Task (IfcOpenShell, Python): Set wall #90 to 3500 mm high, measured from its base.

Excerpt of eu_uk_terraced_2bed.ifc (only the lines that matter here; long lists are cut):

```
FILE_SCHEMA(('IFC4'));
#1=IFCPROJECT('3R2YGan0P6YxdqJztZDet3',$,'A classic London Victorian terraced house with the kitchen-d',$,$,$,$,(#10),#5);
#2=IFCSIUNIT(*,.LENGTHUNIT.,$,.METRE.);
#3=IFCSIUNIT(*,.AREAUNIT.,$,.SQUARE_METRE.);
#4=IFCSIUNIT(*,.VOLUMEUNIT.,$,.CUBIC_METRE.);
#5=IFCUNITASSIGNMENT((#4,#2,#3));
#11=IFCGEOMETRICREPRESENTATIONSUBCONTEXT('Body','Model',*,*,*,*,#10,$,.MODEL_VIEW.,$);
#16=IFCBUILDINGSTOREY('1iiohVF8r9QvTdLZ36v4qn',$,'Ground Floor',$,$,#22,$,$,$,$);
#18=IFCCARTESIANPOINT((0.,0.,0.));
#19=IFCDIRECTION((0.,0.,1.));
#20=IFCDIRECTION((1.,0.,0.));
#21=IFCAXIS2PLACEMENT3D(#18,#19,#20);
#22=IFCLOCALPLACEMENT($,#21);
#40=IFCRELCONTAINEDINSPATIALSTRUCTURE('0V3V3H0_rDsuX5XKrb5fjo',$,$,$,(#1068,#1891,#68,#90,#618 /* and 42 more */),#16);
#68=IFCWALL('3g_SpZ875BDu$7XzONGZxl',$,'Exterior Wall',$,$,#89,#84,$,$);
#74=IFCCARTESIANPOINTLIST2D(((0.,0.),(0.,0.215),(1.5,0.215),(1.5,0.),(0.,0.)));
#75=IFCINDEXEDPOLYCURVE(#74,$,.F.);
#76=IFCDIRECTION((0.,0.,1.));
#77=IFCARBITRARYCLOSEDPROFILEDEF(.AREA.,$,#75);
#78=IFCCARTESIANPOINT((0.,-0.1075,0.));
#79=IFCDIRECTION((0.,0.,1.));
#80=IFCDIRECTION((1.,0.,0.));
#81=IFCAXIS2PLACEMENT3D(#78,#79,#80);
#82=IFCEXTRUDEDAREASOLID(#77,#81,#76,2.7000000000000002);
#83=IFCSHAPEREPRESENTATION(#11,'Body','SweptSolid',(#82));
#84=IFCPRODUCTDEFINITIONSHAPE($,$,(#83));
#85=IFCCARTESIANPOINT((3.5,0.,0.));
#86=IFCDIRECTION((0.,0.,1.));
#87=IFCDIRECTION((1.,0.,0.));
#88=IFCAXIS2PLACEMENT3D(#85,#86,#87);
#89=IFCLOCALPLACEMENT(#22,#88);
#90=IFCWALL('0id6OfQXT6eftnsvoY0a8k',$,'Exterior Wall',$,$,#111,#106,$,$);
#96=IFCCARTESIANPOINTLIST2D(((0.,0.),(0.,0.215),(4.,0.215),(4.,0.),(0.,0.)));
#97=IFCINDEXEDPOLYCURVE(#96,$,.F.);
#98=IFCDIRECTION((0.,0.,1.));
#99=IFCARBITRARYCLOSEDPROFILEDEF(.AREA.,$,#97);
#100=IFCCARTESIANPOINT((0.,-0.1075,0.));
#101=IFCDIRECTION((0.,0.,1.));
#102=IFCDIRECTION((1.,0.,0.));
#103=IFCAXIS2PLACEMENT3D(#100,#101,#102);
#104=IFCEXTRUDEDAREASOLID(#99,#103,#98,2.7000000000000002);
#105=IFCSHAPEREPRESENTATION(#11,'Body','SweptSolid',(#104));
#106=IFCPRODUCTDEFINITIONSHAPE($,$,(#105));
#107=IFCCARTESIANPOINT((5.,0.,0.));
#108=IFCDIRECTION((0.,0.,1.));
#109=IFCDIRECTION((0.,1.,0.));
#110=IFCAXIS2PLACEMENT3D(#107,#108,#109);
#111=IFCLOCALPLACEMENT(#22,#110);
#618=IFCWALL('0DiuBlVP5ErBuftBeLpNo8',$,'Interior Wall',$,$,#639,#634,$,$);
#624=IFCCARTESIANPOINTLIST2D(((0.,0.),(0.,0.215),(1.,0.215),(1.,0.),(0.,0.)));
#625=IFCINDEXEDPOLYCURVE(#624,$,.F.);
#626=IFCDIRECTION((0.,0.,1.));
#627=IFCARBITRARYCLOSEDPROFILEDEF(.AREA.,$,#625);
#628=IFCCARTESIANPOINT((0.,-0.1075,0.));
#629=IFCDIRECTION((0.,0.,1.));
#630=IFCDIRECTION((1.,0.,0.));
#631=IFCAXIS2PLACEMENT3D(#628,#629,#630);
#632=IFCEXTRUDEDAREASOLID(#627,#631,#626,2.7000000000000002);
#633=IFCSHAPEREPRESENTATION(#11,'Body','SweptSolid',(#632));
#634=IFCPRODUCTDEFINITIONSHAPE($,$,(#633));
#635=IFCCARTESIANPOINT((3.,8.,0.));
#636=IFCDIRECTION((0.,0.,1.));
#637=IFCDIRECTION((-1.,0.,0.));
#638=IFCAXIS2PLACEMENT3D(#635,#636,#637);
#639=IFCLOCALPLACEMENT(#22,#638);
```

```python
import ifcopenshell
import ifcopenshell.geom
import ifcopenshell.util.representation
import ifcopenshell.util.shape
import ifcopenshell.util.unit

model = ifcopenshell.open("eu_uk_terraced_2bed.ifc")
unit_scale = ifcopenshell.util.unit.calculate_unit_scale(model)
settings = ifcopenshell.geom.settings()


def volume(element):
    """Net volume in cubic metres, openings subtracted."""
    shape = ifcopenshell.geom.create_shape(settings, element)
    return ifcopenshell.util.shape.get_volume(shape.geometry)


wall = model.by_guid("0id6OfQXT6eftnsvoY0a8k")
before = volume(wall)

body = ifcopenshell.util.representation.get_representation(wall, "Model", "Body")
solid = body.Items[0]
old_height = solid.Depth
solid.Depth = 3.5 / unit_scale
after = volume(wall)

print(f"height {old_height:g} -> {solid.Depth:g}, volume {before:.3f} -> {after:.3f} m3")

model.write("eu_uk_terraced_2bed_rev.ifc")
```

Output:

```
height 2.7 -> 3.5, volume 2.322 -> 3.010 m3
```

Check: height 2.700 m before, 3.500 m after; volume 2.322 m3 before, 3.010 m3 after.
